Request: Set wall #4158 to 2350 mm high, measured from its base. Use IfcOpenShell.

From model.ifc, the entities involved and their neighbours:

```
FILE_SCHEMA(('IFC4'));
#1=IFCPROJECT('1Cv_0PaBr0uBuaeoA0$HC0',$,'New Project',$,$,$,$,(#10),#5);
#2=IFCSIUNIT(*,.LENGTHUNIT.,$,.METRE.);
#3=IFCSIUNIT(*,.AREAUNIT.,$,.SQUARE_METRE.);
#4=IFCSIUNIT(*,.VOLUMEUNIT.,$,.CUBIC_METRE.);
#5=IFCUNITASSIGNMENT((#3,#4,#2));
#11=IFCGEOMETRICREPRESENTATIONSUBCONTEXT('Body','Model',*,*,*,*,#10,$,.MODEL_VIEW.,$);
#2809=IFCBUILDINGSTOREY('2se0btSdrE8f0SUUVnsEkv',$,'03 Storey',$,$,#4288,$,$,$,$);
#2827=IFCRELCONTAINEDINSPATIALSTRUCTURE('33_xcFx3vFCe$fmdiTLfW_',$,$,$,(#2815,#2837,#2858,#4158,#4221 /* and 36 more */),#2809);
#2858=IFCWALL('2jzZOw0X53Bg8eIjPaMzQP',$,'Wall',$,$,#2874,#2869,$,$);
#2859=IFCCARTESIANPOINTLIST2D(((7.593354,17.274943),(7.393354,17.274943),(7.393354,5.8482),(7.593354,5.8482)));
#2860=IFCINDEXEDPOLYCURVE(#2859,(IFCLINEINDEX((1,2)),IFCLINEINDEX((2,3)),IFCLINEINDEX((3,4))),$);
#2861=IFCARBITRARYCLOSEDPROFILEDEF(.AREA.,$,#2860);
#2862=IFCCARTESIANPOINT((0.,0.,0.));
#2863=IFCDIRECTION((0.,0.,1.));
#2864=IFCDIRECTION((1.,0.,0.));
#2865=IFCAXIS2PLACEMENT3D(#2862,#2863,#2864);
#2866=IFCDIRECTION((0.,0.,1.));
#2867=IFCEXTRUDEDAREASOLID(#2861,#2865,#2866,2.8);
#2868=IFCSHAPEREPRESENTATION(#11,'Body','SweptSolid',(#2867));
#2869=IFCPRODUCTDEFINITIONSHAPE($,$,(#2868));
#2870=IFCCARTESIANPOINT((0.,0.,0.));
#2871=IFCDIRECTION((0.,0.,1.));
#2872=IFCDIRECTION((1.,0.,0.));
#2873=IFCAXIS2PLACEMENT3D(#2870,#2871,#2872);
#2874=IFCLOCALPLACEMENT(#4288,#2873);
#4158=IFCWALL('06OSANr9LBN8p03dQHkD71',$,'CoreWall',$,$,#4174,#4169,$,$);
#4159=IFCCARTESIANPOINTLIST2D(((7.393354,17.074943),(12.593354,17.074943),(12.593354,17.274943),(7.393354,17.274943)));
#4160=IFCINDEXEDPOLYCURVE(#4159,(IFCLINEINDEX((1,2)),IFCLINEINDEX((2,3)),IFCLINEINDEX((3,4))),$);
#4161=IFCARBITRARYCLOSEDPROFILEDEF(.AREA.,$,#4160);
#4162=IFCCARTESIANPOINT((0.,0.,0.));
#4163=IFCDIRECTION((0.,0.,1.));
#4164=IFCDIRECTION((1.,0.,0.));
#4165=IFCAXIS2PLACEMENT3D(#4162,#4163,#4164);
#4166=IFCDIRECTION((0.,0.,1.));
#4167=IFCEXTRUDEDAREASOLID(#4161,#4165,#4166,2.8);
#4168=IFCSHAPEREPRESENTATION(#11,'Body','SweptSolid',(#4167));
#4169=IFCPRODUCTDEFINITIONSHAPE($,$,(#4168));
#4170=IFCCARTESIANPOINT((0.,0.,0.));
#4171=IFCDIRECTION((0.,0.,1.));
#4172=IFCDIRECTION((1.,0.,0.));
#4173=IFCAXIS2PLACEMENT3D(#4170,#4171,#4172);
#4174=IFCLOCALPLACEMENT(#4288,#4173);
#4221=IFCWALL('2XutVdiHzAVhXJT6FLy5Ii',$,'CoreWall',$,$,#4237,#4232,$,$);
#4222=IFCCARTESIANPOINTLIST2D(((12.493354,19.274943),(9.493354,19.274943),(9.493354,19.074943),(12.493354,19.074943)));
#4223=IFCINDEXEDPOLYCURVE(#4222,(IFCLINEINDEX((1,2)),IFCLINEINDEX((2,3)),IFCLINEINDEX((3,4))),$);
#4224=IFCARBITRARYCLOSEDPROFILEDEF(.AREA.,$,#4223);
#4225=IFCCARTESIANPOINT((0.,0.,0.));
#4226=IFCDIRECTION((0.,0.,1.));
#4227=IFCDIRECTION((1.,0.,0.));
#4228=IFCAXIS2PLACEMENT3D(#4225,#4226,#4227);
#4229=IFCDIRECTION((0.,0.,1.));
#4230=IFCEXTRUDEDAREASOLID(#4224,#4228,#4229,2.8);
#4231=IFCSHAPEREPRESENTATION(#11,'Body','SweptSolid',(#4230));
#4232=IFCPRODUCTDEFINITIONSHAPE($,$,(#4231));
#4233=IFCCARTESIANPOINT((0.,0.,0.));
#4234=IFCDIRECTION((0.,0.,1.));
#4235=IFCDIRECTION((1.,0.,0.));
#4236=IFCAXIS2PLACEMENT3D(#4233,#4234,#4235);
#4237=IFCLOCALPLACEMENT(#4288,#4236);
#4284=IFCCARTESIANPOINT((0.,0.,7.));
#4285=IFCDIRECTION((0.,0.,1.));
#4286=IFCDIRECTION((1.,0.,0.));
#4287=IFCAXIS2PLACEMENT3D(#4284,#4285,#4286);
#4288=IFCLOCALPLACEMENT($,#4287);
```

```python
import ifcopenshell
import ifcopenshell.geom
import ifcopenshell.util.representation
import ifcopenshell.util.shape
import ifcopenshell.util.unit

model = ifcopenshell.open("model.ifc")
unit_scale = ifcopenshell.util.unit.calculate_unit_scale(model)
settings = ifcopenshell.geom.settings()


def volume(element):
    """Net volume in cubic metres, openings subtracted."""
    shape = ifcopenshell.geom.create_shape(settings, element)
    return ifcopenshell.util.shape.get_volume(shape.geometry)


wall = model.by_guid("06OSANr9LBN8p03dQHkD71")
before = volume(wall)

body = ifcopenshell.util.representation.get_representation(wall, "Model", "Body")
solid = body.Items[0]
old_height = solid.Depth
solid.Depth = 2.35 / unit_scale
after = volume(wall)

print(f"height {old_height:g} -> {solid.Depth:g}, volume {before:.3f} -> {after:.3f} m3")

model.write("model_v2.ifc")
```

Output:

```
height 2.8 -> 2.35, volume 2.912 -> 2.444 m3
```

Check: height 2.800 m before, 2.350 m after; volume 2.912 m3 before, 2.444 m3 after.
